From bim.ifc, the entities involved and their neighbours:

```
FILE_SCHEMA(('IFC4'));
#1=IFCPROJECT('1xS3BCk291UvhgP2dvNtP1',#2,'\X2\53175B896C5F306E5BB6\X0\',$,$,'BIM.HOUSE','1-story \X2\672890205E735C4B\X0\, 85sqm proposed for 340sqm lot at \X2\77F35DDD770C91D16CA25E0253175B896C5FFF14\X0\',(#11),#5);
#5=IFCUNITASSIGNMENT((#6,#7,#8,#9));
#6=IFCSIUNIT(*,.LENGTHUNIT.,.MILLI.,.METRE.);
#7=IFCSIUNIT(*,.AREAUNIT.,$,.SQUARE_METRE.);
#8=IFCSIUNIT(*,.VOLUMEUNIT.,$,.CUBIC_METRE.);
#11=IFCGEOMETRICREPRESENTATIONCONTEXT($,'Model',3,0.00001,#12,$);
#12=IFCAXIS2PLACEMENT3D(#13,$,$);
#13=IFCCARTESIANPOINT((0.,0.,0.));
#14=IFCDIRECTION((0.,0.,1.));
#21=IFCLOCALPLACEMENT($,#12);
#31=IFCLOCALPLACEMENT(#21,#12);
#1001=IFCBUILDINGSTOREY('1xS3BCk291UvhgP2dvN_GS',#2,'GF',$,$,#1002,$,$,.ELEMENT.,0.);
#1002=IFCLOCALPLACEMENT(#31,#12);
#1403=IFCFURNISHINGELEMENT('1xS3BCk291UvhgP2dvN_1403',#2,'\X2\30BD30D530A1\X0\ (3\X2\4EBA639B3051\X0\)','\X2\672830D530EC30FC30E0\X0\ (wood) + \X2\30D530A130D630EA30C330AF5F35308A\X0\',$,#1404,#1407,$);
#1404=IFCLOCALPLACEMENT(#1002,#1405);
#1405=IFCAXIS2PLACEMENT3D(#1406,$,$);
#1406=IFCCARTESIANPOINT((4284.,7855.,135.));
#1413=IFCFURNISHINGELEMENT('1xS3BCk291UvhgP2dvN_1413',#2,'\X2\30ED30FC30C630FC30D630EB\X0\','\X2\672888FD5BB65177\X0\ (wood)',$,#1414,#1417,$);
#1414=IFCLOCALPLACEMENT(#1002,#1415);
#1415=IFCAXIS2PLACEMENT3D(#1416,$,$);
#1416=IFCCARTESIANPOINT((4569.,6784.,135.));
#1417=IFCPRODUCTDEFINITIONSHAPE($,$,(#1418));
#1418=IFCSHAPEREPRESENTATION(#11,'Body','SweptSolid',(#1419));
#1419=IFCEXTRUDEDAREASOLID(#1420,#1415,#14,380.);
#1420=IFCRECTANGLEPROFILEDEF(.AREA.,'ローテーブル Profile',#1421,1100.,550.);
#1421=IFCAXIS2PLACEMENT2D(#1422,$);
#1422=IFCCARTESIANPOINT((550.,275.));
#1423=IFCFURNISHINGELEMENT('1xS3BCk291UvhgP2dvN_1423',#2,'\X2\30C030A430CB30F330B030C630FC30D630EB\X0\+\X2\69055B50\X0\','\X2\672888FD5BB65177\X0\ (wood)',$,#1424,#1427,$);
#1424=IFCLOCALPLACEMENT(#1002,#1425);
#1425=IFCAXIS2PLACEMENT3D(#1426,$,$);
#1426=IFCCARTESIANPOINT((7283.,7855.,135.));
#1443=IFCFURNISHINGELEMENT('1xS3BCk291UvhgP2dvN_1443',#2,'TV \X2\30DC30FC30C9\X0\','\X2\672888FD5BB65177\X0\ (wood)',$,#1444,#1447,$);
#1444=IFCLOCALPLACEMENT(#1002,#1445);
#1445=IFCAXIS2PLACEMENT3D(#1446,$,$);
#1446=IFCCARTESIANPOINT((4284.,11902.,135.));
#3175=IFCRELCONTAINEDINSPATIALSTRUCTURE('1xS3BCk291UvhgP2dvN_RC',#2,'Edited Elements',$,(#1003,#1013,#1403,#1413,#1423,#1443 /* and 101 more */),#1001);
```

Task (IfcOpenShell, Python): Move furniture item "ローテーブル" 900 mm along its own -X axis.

```python
import ifcopenshell
import ifcopenshell.api.geometry
import ifcopenshell.util.placement

model = ifcopenshell.open("bim.ifc")

item = model.by_guid("1xS3BCk291UvhgP2dvN_1413")
matrix = ifcopenshell.util.placement.get_local_placement(item.ObjectPlacement)
matrix[:3, 3] -= matrix[:3, 0] * 900.0
ifcopenshell.api.geometry.edit_object_placement(model, product=item, matrix=matrix, is_si=False)

print(ifcopenshell.util.placement.get_local_placement(item.ObjectPlacement).round(3) + 0.0)

model.write("bim_v2.ifc")
```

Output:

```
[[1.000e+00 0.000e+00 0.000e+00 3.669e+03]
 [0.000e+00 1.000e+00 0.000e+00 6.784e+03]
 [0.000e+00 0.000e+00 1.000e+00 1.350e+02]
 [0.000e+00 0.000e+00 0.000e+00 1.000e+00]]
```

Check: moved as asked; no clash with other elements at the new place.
